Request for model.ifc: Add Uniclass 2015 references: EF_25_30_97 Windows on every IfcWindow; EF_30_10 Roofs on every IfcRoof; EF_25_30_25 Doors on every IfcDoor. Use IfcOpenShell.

First a look at what the model holds.

```python
import ifcopenshell

model = ifcopenshell.open("model.ifc")
print(model.schema)
print("classifications:", [c.Name for c in model.by_type("IfcClassification")])
for ifc_class in ("IfcDoor", "IfcRoof", "IfcStair", "IfcWall", "IfcWindow"):
    print(ifc_class, len(model.by_type(ifc_class)))
```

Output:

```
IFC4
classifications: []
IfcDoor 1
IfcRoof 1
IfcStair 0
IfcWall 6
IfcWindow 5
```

```python
import ifcopenshell
import ifcopenshell.api.classification

model = ifcopenshell.open("model.ifc")

system = ifcopenshell.api.classification.add_classification(model, classification="Uniclass 2015")

codes = {
    "IfcWindow": ("EF_25_30_97", "Windows"),
    "IfcRoof": ("EF_30_10", "Roofs"),
    "IfcDoor": ("EF_25_30_25", "Doors"),
}
for ifc_class, (code, name) in codes.items():
    products = model.by_type(ifc_class)
    ifcopenshell.api.classification.add_reference(
        model, products=products, classification=system, identification=code, name=name
    )
    print(code, len(products))

model.write("model_rev.ifc")
```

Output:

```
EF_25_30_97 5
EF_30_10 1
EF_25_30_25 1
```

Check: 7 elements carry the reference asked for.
